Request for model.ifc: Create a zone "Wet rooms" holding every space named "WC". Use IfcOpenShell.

First a look at what the model holds.

```python
import ifcopenshell

model = ifcopenshell.open("model.ifc")
print(model.schema)
seen = {}
for space in model.by_type("IfcSpace"):
    seen[space.LongName] = seen.get(space.LongName, 0) + 1
for name, count in sorted(seen.items(), key=str):
    print(count, "x", name)
print("zones:", [z.Name for z in model.by_type("IfcZone")][:20])
```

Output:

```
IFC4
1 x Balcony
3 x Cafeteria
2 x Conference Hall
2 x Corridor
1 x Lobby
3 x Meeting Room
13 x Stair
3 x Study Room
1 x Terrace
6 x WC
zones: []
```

```python
import ifcopenshell
import ifcopenshell.api.group
import ifcopenshell.api.root

model = ifcopenshell.open("model.ifc")

names = {"WC"}
spaces = [s for s in model.by_type("IfcSpace") if s.LongName in names]

zone = ifcopenshell.api.root.create_entity(model, ifc_class="IfcZone", name="Wet rooms")
ifcopenshell.api.group.assign_group(model, products=spaces, group=zone)
print(len(spaces), "spaces in", zone.Name)

model.write("model_v2.ifc")
```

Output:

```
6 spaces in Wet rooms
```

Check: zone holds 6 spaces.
